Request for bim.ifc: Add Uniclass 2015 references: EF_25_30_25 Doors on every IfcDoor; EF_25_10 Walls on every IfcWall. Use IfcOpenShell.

First a look at what the model holds.

```python
import ifcopenshell

model = ifcopenshell.open("bim.ifc")
print(model.schema)
print("classifications:", [c.Name for c in model.by_type("IfcClassification")])
for ifc_class in ("IfcDoor", "IfcRoof", "IfcStair", "IfcWall", "IfcWindow"):
    print(ifc_class, len(model.by_type(ifc_class)))
```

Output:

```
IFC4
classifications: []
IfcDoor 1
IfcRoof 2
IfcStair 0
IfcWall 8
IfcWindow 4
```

```python
import ifcopenshell
import ifcopenshell.api.classification

model = ifcopenshell.open("bim.ifc")

system = ifcopenshell.api.classification.add_classification(model, classification="Uniclass 2015")

codes = {
    "IfcDoor": ("EF_25_30_25", "Doors"),
    "IfcWall": ("EF_25_10", "Walls"),
}
for ifc_class, (code, name) in codes.items():
    products = model.by_type(ifc_class)
    ifcopenshell.api.classification.add_reference(
        model, products=products, classification=system, identification=code, name=name
    )
    print(code, len(products))

model.write("bim_edited.ifc")
```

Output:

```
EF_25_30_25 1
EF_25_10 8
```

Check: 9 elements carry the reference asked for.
